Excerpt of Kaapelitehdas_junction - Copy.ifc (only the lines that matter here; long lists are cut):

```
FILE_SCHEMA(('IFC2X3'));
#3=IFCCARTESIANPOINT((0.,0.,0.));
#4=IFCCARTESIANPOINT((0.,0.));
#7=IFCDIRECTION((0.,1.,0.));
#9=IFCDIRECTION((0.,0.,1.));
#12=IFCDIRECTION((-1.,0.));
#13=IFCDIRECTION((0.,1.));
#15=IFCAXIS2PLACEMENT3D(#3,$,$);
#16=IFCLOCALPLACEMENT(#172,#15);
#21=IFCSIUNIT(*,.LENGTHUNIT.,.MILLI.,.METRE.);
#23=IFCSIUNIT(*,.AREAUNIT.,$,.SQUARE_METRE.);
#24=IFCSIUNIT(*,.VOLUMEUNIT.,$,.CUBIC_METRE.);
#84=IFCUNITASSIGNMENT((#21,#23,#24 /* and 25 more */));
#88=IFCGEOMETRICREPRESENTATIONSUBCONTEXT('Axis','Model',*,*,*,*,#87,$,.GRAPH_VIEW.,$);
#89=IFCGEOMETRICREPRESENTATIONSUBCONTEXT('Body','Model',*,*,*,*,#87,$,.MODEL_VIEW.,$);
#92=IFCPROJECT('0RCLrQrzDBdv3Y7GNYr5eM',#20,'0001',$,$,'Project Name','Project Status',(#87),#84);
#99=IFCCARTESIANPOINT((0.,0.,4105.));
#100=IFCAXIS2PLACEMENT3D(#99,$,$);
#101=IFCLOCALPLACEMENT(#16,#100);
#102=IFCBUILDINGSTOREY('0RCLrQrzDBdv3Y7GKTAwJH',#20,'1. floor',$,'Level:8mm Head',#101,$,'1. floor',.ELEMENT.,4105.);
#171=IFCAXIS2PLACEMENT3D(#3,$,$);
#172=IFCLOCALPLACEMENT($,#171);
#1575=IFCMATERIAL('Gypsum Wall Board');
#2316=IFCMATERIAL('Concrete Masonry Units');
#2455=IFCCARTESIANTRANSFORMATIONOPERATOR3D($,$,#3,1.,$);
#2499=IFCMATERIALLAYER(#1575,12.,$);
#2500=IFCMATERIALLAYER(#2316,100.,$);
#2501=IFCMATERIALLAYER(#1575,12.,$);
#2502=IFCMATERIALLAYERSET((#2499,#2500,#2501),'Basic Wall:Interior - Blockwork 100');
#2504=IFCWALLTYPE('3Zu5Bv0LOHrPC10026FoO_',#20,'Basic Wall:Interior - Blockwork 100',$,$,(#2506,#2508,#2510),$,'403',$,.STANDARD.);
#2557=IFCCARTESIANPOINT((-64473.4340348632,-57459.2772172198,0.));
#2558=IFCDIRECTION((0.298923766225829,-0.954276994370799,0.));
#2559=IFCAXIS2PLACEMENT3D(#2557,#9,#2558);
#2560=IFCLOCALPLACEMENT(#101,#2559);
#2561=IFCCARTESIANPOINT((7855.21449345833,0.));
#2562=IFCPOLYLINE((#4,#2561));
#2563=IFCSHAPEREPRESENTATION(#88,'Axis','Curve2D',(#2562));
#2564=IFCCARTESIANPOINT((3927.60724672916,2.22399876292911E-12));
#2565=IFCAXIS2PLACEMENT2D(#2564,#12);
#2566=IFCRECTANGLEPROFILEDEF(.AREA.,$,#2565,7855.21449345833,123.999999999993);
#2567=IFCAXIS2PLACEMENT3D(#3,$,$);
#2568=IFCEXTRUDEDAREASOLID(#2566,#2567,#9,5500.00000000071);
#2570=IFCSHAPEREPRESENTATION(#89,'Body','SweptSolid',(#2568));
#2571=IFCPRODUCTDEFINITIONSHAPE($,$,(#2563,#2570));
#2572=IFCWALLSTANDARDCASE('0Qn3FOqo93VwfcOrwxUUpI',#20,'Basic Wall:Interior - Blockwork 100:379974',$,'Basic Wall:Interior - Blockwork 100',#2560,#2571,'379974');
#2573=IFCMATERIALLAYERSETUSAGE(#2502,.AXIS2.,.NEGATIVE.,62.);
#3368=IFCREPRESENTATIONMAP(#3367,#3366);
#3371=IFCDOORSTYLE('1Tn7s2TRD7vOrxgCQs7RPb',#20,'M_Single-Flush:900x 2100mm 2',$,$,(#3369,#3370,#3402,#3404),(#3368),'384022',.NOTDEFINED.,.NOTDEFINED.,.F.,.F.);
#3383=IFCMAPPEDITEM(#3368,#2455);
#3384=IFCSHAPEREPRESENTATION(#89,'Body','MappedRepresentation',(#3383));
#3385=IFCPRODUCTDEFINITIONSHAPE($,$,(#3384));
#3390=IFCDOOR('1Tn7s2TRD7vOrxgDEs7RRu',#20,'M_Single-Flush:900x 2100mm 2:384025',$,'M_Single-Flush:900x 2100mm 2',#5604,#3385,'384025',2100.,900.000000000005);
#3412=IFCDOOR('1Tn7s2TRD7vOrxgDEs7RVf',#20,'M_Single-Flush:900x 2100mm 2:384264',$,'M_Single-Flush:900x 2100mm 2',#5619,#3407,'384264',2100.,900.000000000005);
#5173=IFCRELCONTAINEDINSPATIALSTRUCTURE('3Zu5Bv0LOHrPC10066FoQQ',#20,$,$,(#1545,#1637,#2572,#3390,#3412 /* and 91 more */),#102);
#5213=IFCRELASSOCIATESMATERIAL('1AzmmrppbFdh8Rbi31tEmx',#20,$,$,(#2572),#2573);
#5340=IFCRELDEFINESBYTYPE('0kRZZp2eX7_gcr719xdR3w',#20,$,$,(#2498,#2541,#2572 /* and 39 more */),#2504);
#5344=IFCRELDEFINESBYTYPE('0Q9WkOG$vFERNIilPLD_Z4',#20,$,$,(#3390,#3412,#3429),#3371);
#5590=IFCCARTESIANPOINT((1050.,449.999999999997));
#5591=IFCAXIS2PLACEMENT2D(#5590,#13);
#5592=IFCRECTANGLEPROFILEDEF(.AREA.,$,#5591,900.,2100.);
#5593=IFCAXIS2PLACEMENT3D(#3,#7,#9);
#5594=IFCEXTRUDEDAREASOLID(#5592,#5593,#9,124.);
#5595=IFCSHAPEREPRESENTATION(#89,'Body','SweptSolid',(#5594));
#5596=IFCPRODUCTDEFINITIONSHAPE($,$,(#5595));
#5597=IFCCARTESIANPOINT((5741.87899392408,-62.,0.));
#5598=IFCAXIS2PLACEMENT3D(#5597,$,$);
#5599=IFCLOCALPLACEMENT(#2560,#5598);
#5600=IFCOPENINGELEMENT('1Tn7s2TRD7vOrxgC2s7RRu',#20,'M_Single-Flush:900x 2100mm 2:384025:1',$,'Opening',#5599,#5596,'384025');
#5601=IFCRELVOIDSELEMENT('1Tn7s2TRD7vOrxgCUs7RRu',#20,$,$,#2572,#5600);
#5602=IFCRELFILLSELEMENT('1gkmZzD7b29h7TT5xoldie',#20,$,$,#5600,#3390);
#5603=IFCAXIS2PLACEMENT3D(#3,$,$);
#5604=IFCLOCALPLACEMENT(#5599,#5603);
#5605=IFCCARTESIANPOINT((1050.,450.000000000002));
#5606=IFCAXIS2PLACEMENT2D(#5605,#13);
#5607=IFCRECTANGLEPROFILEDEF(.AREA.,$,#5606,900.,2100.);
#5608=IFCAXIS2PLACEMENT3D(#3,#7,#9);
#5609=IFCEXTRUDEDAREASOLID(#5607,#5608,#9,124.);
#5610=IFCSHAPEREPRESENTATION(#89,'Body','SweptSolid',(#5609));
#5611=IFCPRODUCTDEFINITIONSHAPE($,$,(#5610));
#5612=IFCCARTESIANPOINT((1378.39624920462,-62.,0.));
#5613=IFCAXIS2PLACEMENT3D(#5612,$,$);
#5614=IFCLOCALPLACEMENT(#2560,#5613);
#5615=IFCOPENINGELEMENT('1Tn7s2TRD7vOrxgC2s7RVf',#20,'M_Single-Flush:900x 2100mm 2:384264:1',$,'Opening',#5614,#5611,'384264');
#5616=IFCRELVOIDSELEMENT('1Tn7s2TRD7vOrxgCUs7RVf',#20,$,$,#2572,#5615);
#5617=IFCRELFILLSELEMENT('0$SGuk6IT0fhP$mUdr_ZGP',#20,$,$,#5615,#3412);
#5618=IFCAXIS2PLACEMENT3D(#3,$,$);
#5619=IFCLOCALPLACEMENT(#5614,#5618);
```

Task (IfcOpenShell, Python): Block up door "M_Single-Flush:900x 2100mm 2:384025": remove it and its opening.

```python
import ifcopenshell
import ifcopenshell.api.feature
import ifcopenshell.api.root
import ifcopenshell.geom
import ifcopenshell.util.shape

model = ifcopenshell.open("Kaapelitehdas_junction - Copy.ifc")
settings = ifcopenshell.geom.settings()


def volume(element):
    """Net volume in cubic metres, openings subtracted."""
    shape = ifcopenshell.geom.create_shape(settings, element)
    return ifcopenshell.util.shape.get_volume(shape.geometry)


door = model.by_guid("1Tn7s2TRD7vOrxgDEs7RRu")
opening = door.FillsVoids[0].RelatingOpeningElement
wall = opening.VoidsElements[0].RelatingBuildingElement
before = volume(wall)

ifcopenshell.api.root.remove_product(model, product=door)
ifcopenshell.api.feature.remove_feature(model, feature=opening)

after = volume(wall)

print(f"wall volume {before:.3f} -> {after:.3f} m3")

model.write("Kaapelitehdas_junction - Copy-out.ifc")
```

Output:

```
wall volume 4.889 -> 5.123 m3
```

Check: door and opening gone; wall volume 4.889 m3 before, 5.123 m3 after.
